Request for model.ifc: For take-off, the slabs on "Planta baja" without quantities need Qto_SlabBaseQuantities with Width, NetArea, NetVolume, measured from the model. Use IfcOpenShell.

First a look at what the model holds.

```python
import ifcopenshell
import ifcopenshell.util.element
import ifcopenshell.util.unit

model = ifcopenshell.open("model.ifc")
print(model.schema)
for unit_type in ("LENGTHUNIT", "AREAUNIT", "VOLUMEUNIT"):
    print(unit_type, ifcopenshell.util.unit.calculate_unit_scale(model, unit_type))
storey = next(s for s in model.by_type("IfcBuildingStorey") if s.Name == "Planta baja")
slabs = [e for e in ifcopenshell.util.element.get_decomposition(storey) if e.is_a("IfcSlab")]
for e in sorted(slabs, key=lambda e: e.id()):
    print(e.id(), e.is_a(), e.Name, list(ifcopenshell.util.element.get_psets(e, qtos_only=True)), sep=" | ")
```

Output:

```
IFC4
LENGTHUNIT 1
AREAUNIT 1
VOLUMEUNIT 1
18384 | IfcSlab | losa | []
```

```python
import ifcopenshell
import ifcopenshell.api.pset
import ifcopenshell.geom
import ifcopenshell.util.element
import ifcopenshell.util.shape
import ifcopenshell.util.unit

model = ifcopenshell.open("model.ifc")
unit_scale = ifcopenshell.util.unit.calculate_unit_scale(model)
area_scale = ifcopenshell.util.unit.calculate_unit_scale(model, "AREAUNIT")
volume_scale = ifcopenshell.util.unit.calculate_unit_scale(model, "VOLUMEUNIT")
settings = ifcopenshell.geom.settings()

storey = next(s for s in model.by_type("IfcBuildingStorey") if s.Name == "Planta baja")
slabs = [e for e in ifcopenshell.util.element.get_decomposition(storey) if e.is_a("IfcSlab")]

for e in sorted(slabs, key=lambda e: e.id()):
    if ifcopenshell.util.element.get_psets(e, qtos_only=True, should_inherit=False):
        continue
    # Geometry comes back in metres, in the element's own axes.
    shape = ifcopenshell.geom.create_shape(settings, e)
    values = {
        "Width": ifcopenshell.util.shape.get_z(shape.geometry) / unit_scale,
        "NetArea": ifcopenshell.util.shape.get_footprint_area(shape.geometry) / area_scale,
        "NetVolume": ifcopenshell.util.shape.get_volume(shape.geometry) / volume_scale,
    }
    qto = ifcopenshell.api.pset.add_qto(model, product=e, name="Qto_SlabBaseQuantities")
    ifcopenshell.api.pset.edit_qto(model, qto=qto, properties=values)
    print(e.id(), {k: round(v, 3) for k, v in values.items()})

model.write("model_v2.ifc")
```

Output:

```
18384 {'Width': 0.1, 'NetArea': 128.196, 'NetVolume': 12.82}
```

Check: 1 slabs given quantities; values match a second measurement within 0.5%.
